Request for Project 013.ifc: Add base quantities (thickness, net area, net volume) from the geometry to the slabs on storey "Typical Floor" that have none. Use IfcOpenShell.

First a look at what the model holds.

```python
import ifcopenshell
import ifcopenshell.util.element
import ifcopenshell.util.unit

model = ifcopenshell.open("Project 013.ifc")
print(model.schema)
for unit_type in ("LENGTHUNIT", "AREAUNIT", "VOLUMEUNIT"):
    print(unit_type, ifcopenshell.util.unit.calculate_unit_scale(model, unit_type))
storey = next(s for s in model.by_type("IfcBuildingStorey") if s.Name == "Typical Floor")
slabs = [e for e in ifcopenshell.util.element.get_decomposition(storey) if e.is_a("IfcSlab")]
for e in sorted(slabs, key=lambda e: e.id()):
    print(e.id(), e.is_a(), e.Name, list(ifcopenshell.util.element.get_psets(e, qtos_only=True)), sep=" | ")
```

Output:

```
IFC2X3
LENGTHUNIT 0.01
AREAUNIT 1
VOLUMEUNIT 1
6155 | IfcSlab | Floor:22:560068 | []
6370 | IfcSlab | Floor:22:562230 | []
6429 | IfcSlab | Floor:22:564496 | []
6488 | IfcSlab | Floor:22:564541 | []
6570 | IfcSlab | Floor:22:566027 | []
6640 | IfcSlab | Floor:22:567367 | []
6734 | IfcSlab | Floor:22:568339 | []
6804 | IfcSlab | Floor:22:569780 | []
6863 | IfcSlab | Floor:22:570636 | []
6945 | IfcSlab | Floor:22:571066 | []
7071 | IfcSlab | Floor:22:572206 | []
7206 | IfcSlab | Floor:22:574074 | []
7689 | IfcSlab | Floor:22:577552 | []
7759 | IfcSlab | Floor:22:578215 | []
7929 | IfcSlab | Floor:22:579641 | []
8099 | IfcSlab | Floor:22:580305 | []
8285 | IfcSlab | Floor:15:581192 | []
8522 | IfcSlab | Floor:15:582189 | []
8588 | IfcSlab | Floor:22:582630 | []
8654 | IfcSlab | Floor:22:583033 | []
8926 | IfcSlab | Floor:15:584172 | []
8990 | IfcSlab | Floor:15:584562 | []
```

```python
import ifcopenshell
import ifcopenshell.api.pset
import ifcopenshell.geom
import ifcopenshell.util.element
import ifcopenshell.util.shape
import ifcopenshell.util.unit

model = ifcopenshell.open("Project 013.ifc")
unit_scale = ifcopenshell.util.unit.calculate_unit_scale(model)
area_scale = ifcopenshell.util.unit.calculate_unit_scale(model, "AREAUNIT")
volume_scale = ifcopenshell.util.unit.calculate_unit_scale(model, "VOLUMEUNIT")
settings = ifcopenshell.geom.settings()

storey = next(s for s in model.by_type("IfcBuildingStorey") if s.Name == "Typical Floor")
slabs = [e for e in ifcopenshell.util.element.get_decomposition(storey) if e.is_a("IfcSlab")]

for e in sorted(slabs, key=lambda e: e.id()):
    if ifcopenshell.util.element.get_psets(e, qtos_only=True, should_inherit=False):
        continue
    # Geometry comes back in metres, in the element's own axes.
    shape = ifcopenshell.geom.create_shape(settings, e)
    values = {
        "Width": ifcopenshell.util.shape.get_z(shape.geometry) / unit_scale,
        "NetArea": ifcopenshell.util.shape.get_footprint_area(shape.geometry) / area_scale,
        "NetVolume": ifcopenshell.util.shape.get_volume(shape.geometry) / volume_scale,
    }
    qto = ifcopenshell.api.pset.add_qto(model, product=e, name="BaseQuantities")
    ifcopenshell.api.pset.edit_qto(model, qto=qto, properties=values)
    print(e.id(), {k: round(v, 3) for k, v in values.items()})

model.write("Project 013_edited.ifc")
```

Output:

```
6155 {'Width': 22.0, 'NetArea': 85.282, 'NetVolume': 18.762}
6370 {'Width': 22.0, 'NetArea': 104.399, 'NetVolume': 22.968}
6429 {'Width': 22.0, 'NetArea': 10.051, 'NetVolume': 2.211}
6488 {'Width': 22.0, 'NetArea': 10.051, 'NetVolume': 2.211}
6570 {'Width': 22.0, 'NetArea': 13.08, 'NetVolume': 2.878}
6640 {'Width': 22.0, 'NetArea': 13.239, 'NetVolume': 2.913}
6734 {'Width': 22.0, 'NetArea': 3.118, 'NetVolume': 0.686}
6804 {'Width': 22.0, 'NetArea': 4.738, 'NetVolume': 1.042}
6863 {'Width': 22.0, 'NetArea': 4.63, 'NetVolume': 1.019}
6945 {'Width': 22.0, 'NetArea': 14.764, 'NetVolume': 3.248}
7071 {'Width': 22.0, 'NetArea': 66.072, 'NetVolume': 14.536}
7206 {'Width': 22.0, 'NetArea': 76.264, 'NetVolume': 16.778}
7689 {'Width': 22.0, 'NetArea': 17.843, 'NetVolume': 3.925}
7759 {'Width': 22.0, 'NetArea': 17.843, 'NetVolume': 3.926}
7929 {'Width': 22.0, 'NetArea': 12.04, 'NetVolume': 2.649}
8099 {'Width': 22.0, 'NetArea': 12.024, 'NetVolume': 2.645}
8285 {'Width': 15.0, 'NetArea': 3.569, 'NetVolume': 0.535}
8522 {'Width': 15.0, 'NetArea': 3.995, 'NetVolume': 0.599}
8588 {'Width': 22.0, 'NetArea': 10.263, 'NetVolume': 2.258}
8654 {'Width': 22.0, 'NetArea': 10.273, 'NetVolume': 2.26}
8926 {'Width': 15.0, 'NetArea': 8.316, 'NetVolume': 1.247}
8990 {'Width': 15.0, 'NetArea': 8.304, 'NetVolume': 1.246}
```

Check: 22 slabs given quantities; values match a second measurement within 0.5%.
